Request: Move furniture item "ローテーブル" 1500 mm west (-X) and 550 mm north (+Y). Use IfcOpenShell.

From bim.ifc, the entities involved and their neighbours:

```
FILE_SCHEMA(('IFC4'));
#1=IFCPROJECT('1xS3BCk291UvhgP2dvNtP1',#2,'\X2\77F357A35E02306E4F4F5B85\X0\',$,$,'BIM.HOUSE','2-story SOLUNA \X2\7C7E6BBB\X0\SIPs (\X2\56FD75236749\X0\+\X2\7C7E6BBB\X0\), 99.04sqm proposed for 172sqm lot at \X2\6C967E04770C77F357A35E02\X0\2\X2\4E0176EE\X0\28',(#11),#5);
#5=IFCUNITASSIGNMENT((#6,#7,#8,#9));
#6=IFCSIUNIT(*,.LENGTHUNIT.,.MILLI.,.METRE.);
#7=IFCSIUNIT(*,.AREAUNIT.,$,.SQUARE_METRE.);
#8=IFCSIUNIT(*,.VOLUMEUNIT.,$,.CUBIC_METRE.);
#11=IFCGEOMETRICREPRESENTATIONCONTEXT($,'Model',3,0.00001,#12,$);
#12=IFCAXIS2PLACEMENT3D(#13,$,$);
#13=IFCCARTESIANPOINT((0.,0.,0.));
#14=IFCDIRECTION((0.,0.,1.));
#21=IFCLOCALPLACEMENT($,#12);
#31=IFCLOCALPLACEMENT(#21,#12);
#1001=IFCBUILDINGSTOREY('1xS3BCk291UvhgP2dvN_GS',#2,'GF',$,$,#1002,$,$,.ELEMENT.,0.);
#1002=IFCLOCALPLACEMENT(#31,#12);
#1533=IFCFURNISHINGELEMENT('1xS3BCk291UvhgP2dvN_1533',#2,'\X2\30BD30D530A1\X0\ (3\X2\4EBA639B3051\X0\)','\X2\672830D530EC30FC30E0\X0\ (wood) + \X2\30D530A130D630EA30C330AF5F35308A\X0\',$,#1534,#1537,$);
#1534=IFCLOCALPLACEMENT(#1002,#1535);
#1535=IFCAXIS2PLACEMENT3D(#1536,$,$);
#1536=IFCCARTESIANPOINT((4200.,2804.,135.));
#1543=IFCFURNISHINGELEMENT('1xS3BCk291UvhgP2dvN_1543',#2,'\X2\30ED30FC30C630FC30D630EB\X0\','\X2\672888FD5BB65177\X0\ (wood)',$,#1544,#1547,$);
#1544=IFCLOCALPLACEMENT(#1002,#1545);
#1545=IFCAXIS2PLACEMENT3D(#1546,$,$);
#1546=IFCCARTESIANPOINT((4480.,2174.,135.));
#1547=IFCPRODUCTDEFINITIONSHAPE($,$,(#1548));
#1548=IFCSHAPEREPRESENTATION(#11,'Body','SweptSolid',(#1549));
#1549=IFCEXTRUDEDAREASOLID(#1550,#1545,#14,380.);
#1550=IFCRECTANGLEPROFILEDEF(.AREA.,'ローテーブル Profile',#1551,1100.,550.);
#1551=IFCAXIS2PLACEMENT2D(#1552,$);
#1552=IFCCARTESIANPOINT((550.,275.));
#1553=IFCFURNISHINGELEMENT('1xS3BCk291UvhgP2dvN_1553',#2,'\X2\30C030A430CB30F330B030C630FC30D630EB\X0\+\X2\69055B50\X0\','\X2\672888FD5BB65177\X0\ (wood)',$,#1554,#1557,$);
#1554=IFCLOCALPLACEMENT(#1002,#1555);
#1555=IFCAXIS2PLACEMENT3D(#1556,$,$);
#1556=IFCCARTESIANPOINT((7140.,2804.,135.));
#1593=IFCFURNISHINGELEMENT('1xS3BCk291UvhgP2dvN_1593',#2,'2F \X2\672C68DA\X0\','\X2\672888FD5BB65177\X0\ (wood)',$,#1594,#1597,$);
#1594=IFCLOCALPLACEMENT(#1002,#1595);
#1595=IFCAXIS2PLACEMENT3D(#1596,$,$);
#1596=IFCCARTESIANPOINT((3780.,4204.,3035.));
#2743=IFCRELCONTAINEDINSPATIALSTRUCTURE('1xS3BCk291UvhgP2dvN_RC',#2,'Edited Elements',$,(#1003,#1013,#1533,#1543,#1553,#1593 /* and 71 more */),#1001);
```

```python
import ifcopenshell
import ifcopenshell.api.geometry
import ifcopenshell.util.placement
import ifcopenshell.util.unit

model = ifcopenshell.open("bim.ifc")
unit_scale = ifcopenshell.util.unit.calculate_unit_scale(model)

item = model.by_guid("1xS3BCk291UvhgP2dvN_1543")
matrix = ifcopenshell.util.placement.get_local_placement(item.ObjectPlacement)
matrix[0, 3] -= 1.5 / unit_scale
matrix[1, 3] += 0.55 / unit_scale
ifcopenshell.api.geometry.edit_object_placement(model, product=item, matrix=matrix, is_si=False)

print(ifcopenshell.util.placement.get_local_placement(item.ObjectPlacement).round(3) + 0.0)

model.write("bim_edited.ifc")
```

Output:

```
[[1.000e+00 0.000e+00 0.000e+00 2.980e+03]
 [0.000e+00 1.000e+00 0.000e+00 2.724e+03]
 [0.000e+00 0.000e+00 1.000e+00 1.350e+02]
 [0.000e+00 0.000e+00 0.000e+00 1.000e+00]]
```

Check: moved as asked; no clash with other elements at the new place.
